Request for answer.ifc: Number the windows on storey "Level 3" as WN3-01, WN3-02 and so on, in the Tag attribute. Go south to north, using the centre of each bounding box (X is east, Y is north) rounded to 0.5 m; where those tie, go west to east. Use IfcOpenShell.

First a look at what the model holds.

```python
import ifcopenshell
import ifcopenshell.util.element
import ifcopenshell.util.placement

model = ifcopenshell.open("answer.ifc")
print(model.schema)
storey = next(s for s in model.by_type("IfcBuildingStorey") if s.Name == "Level 3")
windows = [e for e in ifcopenshell.util.element.get_decomposition(storey) if e.is_a("IfcWindow")]
for e in sorted(windows, key=lambda e: e.id()):
    origin = ifcopenshell.util.placement.get_local_placement(e.ObjectPlacement)[:3, 3]
    print(e.id(), e.Tag, e.Name, origin.round(2) + 0.0, sep=" | ")
```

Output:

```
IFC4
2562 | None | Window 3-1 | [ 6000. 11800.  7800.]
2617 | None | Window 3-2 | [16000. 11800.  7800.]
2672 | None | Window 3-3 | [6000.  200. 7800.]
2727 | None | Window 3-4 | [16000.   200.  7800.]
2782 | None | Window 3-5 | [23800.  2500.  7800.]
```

```python
import ifcopenshell
import ifcopenshell.geom
import ifcopenshell.util.element
import ifcopenshell.util.shape

model = ifcopenshell.open("answer.ifc")
settings = ifcopenshell.geom.settings()
settings.set("use-world-coords", True)


def centre(element):
    shape = ifcopenshell.geom.create_shape(settings, element)
    return ifcopenshell.util.shape.get_bbox_centroid(shape.geometry)


storey = next(s for s in model.by_type("IfcBuildingStorey") if s.Name == "Level 3")
windows = [e for e in ifcopenshell.util.element.get_decomposition(storey) if e.is_a("IfcWindow")]

# Insertion points can sit at a corner or the storey origin, so sort by the geometry (in metres).
centres = {e: centre(e) for e in windows}
windows.sort(key=lambda e: (round(centres[e][1] / 0.5), centres[e][0]))

for i, e in enumerate(windows, start=1):
    number = f"WN3-{i:02d}"
    e.Tag = number
    print(e.id(), number)

model.write("answer-out.ifc")
```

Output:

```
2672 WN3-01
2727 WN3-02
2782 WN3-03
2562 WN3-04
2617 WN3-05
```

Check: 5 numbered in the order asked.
